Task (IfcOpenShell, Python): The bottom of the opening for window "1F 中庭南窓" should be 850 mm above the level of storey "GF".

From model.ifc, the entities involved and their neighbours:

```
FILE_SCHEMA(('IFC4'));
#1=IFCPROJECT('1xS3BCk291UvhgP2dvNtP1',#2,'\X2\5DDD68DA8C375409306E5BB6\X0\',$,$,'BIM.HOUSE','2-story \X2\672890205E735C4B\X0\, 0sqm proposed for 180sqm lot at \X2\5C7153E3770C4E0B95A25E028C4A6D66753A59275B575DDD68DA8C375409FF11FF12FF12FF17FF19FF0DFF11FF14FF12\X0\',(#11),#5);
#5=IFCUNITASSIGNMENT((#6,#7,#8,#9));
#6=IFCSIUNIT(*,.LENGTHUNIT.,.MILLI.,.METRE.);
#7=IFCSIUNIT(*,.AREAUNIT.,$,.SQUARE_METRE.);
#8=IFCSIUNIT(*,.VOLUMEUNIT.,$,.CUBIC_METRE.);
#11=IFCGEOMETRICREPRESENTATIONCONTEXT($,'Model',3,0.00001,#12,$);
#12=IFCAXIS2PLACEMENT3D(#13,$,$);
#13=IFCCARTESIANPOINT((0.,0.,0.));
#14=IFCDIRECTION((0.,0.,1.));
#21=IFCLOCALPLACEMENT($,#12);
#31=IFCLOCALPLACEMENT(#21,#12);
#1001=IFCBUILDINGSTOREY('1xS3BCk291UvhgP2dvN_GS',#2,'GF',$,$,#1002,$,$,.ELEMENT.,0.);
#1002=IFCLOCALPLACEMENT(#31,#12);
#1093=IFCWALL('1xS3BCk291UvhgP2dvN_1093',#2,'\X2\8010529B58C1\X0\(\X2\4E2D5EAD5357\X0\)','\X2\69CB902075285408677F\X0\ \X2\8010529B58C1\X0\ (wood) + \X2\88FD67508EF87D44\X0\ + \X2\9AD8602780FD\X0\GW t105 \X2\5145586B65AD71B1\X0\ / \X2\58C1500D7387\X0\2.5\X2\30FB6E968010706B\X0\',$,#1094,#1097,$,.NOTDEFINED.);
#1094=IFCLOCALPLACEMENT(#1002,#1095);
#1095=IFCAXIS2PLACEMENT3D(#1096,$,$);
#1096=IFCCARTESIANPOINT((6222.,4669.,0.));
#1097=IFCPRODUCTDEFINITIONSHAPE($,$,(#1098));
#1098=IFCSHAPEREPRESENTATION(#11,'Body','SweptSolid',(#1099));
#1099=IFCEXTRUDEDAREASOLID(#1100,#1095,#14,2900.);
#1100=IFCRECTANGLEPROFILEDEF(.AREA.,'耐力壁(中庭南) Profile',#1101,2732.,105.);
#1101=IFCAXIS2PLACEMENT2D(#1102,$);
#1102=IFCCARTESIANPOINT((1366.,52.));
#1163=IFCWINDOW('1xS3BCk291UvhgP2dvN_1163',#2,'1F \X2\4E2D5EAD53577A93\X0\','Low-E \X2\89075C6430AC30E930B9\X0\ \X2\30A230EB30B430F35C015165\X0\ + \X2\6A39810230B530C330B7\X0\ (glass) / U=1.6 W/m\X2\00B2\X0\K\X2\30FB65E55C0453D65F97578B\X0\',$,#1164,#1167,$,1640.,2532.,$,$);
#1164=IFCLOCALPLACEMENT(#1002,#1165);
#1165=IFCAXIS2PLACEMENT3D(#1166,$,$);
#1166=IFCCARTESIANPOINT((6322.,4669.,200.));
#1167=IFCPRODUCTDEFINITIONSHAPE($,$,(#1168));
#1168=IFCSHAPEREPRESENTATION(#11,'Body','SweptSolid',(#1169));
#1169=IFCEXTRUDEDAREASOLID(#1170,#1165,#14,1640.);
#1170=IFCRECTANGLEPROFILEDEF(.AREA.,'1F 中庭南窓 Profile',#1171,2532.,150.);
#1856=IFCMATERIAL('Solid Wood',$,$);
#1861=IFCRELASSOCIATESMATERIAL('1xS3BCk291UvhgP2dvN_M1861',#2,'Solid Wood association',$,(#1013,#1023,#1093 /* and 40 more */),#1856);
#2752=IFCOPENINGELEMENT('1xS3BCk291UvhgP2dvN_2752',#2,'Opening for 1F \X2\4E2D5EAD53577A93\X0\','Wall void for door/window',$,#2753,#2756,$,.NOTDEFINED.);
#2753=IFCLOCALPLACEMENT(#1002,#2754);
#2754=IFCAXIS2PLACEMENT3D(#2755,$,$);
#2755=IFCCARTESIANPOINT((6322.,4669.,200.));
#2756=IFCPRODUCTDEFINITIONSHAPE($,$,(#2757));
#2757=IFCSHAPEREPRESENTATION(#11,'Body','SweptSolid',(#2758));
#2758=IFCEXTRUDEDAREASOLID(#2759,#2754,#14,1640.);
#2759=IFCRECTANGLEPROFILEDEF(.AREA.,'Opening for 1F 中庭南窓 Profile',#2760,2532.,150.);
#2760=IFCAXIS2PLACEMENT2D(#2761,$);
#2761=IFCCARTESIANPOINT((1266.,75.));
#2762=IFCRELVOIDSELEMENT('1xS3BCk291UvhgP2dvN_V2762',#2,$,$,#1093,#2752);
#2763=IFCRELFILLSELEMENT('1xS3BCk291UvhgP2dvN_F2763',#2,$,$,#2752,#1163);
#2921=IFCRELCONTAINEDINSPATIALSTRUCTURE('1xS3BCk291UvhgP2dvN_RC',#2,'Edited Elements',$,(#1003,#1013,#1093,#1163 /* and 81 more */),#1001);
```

```python
import numpy as np
import ifcopenshell
import ifcopenshell.api.geometry
import ifcopenshell.geom
import ifcopenshell.util.element
import ifcopenshell.util.placement
import ifcopenshell.util.shape
import ifcopenshell.util.unit

model = ifcopenshell.open("model.ifc")
unit_scale = ifcopenshell.util.unit.calculate_unit_scale(model)

window = model.by_guid("1xS3BCk291UvhgP2dvN_1163")
opening = window.FillsVoids[0].RelatingOpeningElement
storey = ifcopenshell.util.element.get_container(window, ifc_class="IfcBuildingStorey")
level = ifcopenshell.util.placement.get_local_placement(storey.ObjectPlacement)[2, 3]

# The opening's origin need not be at the sill, so measure its lowest point.
shape = ifcopenshell.geom.create_shape(ifcopenshell.geom.settings(), opening)
bottom = ifcopenshell.util.shape.get_shape_bottom_elevation(shape, shape.geometry) / unit_scale
dz = level + 850.0 - bottom

shift = np.array([0.0, 0.0, dz])
# The window is not placed relative to its opening, so move both.
for product in (opening, window):
    matrix = ifcopenshell.util.placement.get_local_placement(product.ObjectPlacement)
    matrix[:3, 3] += shift
    ifcopenshell.api.geometry.edit_object_placement(model, product=product, matrix=matrix, is_si=False)

print(f"moved by {dz * unit_scale:+.3f} m")

model.write("model_v2.ifc")
```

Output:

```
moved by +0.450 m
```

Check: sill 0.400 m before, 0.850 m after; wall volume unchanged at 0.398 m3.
